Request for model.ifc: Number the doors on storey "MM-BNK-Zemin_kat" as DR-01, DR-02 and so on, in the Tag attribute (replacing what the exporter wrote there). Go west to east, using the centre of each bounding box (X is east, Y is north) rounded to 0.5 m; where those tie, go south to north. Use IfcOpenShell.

First a look at what the model holds.

```python
import ifcopenshell
import ifcopenshell.util.element
import ifcopenshell.util.placement

model = ifcopenshell.open("model.ifc")
print(model.schema)
storey = next(s for s in model.by_type("IfcBuildingStorey") if s.Name == "MM-BNK-Zemin_kat")
doors = [e for e in ifcopenshell.util.element.get_decomposition(storey) if e.is_a("IfcDoor")]
for e in sorted(doors, key=lambda e: e.id()):
    origin = ifcopenshell.util.placement.get_local_placement(e.ObjectPlacement)[:3, 3]
    print(e.id(), e.Tag, e.Name, origin.round(2) + 0.0, sep=" | ")
```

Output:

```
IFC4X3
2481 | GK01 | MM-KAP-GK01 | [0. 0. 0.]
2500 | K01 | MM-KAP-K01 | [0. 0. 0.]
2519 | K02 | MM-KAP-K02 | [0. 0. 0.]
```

```python
import ifcopenshell
import ifcopenshell.geom
import ifcopenshell.util.element
import ifcopenshell.util.shape

model = ifcopenshell.open("model.ifc")
settings = ifcopenshell.geom.settings()
settings.set("use-world-coords", True)


def centre(element):
    shape = ifcopenshell.geom.create_shape(settings, element)
    return ifcopenshell.util.shape.get_bbox_centroid(shape.geometry)


storey = next(s for s in model.by_type("IfcBuildingStorey") if s.Name == "MM-BNK-Zemin_kat")
doors = [e for e in ifcopenshell.util.element.get_decomposition(storey) if e.is_a("IfcDoor")]

# Insertion points can sit at a corner or the storey origin, so sort by the geometry (in metres).
centres = {e: centre(e) for e in doors}
doors.sort(key=lambda e: (round(centres[e][0] / 0.5), centres[e][1]))

for i, e in enumerate(doors, start=1):
    number = f"DR-{i:02d}"
    e.Tag = number
    print(e.id(), number)

model.write("model_updated.ifc")
```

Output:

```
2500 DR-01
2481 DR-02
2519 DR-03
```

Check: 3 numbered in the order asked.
